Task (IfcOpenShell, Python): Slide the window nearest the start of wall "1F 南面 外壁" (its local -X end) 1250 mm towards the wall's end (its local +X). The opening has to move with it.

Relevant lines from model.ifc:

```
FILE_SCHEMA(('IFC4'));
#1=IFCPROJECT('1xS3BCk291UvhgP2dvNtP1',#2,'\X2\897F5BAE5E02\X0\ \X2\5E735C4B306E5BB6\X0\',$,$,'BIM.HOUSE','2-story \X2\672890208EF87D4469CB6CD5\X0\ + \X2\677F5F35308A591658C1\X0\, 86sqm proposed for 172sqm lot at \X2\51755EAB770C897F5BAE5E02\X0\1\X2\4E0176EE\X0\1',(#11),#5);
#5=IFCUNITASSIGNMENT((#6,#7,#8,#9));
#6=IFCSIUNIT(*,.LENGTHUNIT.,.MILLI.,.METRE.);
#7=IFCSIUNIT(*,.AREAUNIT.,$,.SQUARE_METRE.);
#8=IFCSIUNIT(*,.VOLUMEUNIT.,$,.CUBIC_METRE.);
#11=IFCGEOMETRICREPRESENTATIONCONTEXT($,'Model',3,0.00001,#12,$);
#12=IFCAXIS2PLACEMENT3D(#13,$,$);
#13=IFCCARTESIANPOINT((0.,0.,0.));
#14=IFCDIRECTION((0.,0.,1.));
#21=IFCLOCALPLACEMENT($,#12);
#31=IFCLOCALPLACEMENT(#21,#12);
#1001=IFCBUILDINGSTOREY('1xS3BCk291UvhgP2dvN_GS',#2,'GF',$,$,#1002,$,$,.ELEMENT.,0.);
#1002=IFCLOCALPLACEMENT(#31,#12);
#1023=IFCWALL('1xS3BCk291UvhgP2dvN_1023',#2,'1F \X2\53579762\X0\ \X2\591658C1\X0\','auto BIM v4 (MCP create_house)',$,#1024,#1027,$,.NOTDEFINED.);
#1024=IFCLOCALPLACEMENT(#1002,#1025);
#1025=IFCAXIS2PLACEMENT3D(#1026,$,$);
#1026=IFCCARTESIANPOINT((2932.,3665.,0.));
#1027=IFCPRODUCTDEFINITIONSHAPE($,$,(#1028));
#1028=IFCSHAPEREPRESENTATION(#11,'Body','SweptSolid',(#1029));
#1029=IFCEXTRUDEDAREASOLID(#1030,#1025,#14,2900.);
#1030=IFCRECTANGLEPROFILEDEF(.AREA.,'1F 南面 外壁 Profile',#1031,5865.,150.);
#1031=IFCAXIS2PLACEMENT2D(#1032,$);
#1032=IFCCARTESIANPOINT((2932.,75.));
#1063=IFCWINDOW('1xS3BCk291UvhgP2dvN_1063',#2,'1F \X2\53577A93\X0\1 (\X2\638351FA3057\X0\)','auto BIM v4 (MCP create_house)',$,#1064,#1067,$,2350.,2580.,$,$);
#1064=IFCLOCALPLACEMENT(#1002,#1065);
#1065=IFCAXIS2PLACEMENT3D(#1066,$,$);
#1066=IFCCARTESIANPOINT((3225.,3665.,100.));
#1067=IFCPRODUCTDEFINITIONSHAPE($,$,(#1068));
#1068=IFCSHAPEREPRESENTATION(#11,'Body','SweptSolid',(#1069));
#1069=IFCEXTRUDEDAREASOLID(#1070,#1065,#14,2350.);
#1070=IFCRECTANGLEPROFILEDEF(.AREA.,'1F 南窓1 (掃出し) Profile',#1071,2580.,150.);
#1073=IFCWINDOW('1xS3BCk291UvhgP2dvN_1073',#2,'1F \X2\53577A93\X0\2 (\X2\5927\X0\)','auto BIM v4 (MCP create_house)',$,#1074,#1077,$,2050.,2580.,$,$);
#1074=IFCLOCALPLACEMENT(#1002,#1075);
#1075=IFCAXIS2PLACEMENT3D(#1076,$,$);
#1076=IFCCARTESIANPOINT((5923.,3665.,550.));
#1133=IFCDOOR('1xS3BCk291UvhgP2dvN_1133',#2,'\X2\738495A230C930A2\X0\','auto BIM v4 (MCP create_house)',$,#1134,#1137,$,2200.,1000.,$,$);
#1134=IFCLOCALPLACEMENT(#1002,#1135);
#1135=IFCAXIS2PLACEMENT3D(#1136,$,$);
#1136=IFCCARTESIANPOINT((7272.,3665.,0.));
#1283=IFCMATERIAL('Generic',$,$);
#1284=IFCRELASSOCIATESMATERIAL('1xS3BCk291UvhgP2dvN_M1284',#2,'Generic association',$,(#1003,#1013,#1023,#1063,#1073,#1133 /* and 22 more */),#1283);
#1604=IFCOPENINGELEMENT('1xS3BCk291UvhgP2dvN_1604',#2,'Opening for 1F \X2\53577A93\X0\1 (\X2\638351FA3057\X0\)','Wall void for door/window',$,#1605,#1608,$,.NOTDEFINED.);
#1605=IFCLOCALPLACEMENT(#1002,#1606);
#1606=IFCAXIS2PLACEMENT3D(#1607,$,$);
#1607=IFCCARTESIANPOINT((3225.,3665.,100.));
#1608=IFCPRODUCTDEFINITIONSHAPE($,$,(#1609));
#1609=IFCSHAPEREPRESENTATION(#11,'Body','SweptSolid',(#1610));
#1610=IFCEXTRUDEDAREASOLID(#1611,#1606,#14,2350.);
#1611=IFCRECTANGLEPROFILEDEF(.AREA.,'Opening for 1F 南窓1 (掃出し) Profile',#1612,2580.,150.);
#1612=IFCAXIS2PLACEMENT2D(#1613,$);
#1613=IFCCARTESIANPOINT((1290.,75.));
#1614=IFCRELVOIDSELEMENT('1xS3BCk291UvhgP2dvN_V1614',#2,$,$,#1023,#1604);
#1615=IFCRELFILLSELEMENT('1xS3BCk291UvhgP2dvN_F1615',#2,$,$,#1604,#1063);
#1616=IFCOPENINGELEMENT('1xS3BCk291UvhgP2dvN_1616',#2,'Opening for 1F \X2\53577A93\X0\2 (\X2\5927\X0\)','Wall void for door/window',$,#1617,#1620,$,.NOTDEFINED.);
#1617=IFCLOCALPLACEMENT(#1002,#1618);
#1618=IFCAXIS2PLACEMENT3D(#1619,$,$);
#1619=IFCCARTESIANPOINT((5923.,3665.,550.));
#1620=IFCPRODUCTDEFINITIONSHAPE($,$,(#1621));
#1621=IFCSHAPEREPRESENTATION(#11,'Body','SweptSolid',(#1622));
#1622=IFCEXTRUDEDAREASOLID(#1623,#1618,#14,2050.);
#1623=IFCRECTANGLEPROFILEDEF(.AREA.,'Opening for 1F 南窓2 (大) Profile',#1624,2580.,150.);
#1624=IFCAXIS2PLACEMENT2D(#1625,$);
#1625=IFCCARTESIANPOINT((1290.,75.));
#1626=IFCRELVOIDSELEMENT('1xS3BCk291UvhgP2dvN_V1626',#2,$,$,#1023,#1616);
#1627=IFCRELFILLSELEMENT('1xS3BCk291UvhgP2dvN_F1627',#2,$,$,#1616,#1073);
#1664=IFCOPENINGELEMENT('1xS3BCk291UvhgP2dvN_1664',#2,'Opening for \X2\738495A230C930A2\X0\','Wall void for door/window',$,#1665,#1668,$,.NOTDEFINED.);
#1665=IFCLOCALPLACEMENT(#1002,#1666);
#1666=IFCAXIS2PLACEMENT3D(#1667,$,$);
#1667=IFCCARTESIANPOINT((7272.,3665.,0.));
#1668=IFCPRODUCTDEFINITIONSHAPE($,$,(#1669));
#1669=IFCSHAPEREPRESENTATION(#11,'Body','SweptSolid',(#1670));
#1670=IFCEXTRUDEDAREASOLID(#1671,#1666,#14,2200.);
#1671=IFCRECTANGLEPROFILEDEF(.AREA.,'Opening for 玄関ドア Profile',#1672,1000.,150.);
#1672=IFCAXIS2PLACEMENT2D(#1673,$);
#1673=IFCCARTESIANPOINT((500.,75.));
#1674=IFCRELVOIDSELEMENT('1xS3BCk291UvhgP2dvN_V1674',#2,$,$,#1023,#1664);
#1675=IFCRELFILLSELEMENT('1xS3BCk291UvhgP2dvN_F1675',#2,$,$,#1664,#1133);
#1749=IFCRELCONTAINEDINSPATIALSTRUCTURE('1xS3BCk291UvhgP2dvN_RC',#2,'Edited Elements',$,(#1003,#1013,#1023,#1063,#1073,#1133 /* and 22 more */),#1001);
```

```python
import ifcopenshell
import ifcopenshell.api.geometry
import ifcopenshell.util.placement
import ifcopenshell.util.unit

model = ifcopenshell.open("model.ifc")
unit_scale = ifcopenshell.util.unit.calculate_unit_scale(model)

window = model.by_guid("1xS3BCk291UvhgP2dvN_1063")
opening = window.FillsVoids[0].RelatingOpeningElement
wall = opening.VoidsElements[0].RelatingBuildingElement

wall_matrix = ifcopenshell.util.placement.get_local_placement(wall.ObjectPlacement)
shift = wall_matrix[:3, 0] * 1.25 / unit_scale
before = ifcopenshell.util.placement.get_local_placement(window.ObjectPlacement)[:3, 3].copy()

# The window is not placed relative to its opening, so move both.
for product in (opening, window):
    matrix = ifcopenshell.util.placement.get_local_placement(product.ObjectPlacement)
    matrix[:3, 3] += shift
    ifcopenshell.api.geometry.edit_object_placement(model, product=product, matrix=matrix, is_si=False)

after = ifcopenshell.util.placement.get_local_placement(window.ObjectPlacement)[:3, 3]
print("window moved by", (after - before).round(3) + 0.0)

model.write("model_rev.ifc")
```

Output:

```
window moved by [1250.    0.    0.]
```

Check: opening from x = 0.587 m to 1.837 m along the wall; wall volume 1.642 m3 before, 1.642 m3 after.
